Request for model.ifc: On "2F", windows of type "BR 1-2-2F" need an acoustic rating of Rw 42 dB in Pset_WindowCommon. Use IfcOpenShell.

First a look at what the model holds.

```python
import ifcopenshell
import ifcopenshell.util.element

model = ifcopenshell.open("model.ifc")
print(model.schema)
storey = next(s for s in model.by_type("IfcBuildingStorey") if s.Name == "2F")
windows = [e for e in ifcopenshell.util.element.get_decomposition(storey) if e.is_a("IfcWindow")]
seen = {}
for e in windows:
    element_type = ifcopenshell.util.element.get_type(e)
    key = (element_type.Name if element_type != e and element_type else None, ifcopenshell.util.element.get_pset(e, "Pset_WindowCommon", "AcousticRating"))
    seen[key] = seen.get(key, 0) + 1
for (name, value), count in sorted(seen.items(), key=str):
    print(count, "x", name, "|", value)
```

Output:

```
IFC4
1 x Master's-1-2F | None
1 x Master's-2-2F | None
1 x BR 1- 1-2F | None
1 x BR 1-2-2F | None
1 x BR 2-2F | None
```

```python
import ifcopenshell
import ifcopenshell.api.pset
import ifcopenshell.util.element

model = ifcopenshell.open("model.ifc")

storey = next(s for s in model.by_type("IfcBuildingStorey") if s.Name == "2F")
windows = [e for e in ifcopenshell.util.element.get_decomposition(storey) if e.is_a("IfcWindow")]

count = 0
for e in windows:
    element_type = ifcopenshell.util.element.get_type(e)
    if element_type in (None, e) or element_type.Name != "BR 1-2-2F":
        continue
    # add_pset returns the element's existing set when there is one.
    pset = ifcopenshell.api.pset.add_pset(model, product=e, name="Pset_WindowCommon")
    ifcopenshell.api.pset.edit_pset(model, pset=pset, properties={"AcousticRating": "Rw 42 dB"})
    count += 1

print(count, "windows updated")

model.write("model_v2.ifc")
```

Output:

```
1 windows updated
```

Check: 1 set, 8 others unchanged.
